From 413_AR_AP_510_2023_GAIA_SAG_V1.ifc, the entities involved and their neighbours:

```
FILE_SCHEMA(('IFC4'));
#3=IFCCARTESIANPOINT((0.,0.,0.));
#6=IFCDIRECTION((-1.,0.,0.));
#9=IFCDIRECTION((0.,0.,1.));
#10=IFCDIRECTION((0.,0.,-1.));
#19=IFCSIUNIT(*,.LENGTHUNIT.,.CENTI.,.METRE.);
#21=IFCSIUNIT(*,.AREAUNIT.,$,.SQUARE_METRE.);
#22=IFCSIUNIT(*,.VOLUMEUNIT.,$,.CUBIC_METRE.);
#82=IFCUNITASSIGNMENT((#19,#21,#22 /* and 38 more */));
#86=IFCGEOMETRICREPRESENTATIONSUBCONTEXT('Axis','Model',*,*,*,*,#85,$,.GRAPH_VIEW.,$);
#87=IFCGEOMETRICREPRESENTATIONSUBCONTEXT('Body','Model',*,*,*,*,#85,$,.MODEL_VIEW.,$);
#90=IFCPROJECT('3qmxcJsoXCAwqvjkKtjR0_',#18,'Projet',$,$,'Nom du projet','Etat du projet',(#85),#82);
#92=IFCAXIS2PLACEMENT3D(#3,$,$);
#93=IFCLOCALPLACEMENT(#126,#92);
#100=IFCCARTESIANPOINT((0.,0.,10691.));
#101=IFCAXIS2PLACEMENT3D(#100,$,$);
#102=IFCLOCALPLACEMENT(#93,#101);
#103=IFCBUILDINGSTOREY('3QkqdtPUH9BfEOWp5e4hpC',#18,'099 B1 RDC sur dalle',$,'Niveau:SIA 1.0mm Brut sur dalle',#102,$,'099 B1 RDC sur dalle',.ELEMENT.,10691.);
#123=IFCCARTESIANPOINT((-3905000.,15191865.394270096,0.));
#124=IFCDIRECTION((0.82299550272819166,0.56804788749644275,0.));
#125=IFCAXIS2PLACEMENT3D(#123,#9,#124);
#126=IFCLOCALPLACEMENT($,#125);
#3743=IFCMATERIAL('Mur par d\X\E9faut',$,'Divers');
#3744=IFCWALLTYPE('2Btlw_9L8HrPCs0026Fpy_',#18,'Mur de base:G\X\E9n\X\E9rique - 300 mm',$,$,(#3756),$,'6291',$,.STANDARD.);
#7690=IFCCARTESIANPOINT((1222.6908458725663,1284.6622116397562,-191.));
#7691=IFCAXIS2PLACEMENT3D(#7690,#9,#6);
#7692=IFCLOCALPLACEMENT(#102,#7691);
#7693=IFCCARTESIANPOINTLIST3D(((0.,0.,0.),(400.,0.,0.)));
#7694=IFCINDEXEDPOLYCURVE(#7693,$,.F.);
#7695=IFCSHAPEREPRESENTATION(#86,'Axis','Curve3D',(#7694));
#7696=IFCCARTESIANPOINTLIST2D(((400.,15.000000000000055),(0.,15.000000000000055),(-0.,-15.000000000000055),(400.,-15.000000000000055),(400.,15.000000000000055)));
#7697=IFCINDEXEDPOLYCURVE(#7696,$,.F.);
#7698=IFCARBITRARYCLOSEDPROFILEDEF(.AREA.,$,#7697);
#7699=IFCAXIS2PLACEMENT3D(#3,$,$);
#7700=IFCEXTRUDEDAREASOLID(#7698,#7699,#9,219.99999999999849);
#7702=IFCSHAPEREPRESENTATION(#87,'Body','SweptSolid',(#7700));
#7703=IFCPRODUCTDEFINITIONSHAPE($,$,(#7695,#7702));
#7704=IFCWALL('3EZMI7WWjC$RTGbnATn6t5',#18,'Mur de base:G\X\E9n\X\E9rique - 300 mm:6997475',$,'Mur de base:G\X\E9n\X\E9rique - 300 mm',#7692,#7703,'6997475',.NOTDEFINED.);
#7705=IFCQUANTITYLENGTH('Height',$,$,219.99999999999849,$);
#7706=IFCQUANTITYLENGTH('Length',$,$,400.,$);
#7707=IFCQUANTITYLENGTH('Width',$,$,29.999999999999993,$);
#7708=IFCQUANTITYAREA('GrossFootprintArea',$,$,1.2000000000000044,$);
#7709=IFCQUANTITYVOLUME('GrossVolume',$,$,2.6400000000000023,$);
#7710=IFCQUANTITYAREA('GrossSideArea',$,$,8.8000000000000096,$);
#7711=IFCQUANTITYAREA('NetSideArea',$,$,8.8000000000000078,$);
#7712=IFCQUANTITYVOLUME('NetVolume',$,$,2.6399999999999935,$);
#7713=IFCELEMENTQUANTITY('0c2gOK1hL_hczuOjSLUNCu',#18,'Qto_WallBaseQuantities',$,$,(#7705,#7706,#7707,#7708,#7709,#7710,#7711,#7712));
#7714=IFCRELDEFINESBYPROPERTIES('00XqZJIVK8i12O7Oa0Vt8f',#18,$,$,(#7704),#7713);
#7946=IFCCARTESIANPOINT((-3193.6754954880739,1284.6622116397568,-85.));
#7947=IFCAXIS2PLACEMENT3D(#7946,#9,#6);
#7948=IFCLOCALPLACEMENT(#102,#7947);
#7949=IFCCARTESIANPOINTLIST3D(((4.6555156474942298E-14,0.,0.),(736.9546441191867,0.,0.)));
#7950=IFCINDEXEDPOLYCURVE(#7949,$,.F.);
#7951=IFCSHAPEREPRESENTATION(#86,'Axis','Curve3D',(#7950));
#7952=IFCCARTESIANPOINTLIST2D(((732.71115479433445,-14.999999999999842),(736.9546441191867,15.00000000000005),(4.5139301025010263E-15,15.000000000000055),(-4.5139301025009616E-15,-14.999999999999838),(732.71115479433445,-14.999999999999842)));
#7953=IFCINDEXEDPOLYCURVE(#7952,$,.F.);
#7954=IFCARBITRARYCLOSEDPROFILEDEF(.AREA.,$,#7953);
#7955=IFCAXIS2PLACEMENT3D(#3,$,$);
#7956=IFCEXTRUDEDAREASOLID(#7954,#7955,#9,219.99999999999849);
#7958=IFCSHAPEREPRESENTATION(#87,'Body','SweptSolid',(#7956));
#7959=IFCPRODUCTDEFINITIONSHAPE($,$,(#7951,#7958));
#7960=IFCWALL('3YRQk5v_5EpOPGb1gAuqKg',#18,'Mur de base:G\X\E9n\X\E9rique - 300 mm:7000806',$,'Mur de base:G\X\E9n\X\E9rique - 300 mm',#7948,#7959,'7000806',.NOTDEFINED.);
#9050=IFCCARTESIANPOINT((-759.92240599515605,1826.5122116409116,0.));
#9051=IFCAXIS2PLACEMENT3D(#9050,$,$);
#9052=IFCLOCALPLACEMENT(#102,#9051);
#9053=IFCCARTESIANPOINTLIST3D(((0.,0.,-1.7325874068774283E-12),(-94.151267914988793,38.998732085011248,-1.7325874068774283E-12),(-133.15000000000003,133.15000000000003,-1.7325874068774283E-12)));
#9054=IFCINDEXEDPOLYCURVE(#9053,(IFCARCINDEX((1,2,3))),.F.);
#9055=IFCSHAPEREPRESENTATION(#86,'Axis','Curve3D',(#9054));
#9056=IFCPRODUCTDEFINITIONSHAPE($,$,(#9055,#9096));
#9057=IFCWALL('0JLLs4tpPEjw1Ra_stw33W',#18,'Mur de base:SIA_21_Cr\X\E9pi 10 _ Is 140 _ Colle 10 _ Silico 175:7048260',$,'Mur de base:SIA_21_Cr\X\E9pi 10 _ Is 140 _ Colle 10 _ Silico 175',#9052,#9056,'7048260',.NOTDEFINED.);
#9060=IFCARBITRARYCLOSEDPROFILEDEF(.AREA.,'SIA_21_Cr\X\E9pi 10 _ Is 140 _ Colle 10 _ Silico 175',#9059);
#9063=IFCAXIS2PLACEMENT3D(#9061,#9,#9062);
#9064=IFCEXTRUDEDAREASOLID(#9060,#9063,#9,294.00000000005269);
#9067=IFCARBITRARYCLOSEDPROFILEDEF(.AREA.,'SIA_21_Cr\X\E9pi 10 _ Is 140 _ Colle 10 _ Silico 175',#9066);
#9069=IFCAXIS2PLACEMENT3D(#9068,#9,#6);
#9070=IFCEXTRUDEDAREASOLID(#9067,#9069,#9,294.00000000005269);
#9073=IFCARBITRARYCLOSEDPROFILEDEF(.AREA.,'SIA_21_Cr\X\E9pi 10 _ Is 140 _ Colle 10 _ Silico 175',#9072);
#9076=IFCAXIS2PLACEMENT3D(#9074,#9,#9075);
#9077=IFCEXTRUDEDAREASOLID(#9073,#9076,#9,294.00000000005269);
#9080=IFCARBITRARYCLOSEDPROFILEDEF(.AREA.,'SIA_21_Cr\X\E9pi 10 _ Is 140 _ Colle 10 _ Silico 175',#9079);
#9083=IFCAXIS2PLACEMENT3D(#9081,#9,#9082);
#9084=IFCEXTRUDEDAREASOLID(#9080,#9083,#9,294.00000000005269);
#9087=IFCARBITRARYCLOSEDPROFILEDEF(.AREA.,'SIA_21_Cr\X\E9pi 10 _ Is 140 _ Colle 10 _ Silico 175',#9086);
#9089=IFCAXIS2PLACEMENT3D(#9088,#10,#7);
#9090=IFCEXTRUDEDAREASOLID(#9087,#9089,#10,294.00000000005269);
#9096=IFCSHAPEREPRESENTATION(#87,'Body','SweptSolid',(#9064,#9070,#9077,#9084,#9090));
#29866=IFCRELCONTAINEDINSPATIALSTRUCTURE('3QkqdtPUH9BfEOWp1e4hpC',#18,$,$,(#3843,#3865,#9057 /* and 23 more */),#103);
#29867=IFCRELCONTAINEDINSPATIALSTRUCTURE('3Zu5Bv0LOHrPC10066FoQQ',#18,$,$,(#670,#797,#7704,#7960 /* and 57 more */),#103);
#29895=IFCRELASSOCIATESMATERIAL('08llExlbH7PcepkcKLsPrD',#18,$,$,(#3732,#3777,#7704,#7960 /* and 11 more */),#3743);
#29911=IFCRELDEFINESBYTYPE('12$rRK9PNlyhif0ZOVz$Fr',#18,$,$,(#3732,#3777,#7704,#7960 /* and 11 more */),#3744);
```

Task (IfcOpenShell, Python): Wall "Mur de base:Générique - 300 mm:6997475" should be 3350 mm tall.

```python
import ifcopenshell
import ifcopenshell.api.pset
import ifcopenshell.geom
import ifcopenshell.util.element
import ifcopenshell.util.representation
import ifcopenshell.util.shape
import ifcopenshell.util.unit

model = ifcopenshell.open("413_AR_AP_510_2023_GAIA_SAG_V1.ifc")
unit_scale = ifcopenshell.util.unit.calculate_unit_scale(model)
area_scale = ifcopenshell.util.unit.calculate_unit_scale(model, "AREAUNIT")
volume_scale = ifcopenshell.util.unit.calculate_unit_scale(model, "VOLUMEUNIT")
settings = ifcopenshell.geom.settings()


def volume(element):
    """Net volume in cubic metres, openings subtracted."""
    shape = ifcopenshell.geom.create_shape(settings, element)
    return ifcopenshell.util.shape.get_volume(shape.geometry)


wall = model.by_guid("3EZMI7WWjC$RTGbnATn6t5")
before = volume(wall)

body = ifcopenshell.util.representation.get_representation(wall, "Model", "Body")
solid = body.Items[0]
old_height = solid.Depth
solid.Depth = 3.35 / unit_scale
after = volume(wall)
thickness = 0.3  # wall thickness in metres

# Update the stored height, areas and volumes.
qto = model.by_id(ifcopenshell.util.element.get_pset(wall, "Qto_WallBaseQuantities", should_inherit=False)["id"])
ifcopenshell.api.pset.edit_qto(model, qto=qto, properties={
    "Height": solid.Depth,
    "GrossVolume": ifcopenshell.util.element.get_pset(wall, "Qto_WallBaseQuantities", "GrossVolume") * solid.Depth / old_height,
    "GrossSideArea": ifcopenshell.util.element.get_pset(wall, "Qto_WallBaseQuantities", "GrossSideArea") * solid.Depth / old_height,
    "NetSideArea": after / thickness / area_scale,
    "NetVolume": after / volume_scale,
})

print(f"height {old_height:g} -> {solid.Depth:g}, volume {before:.3f} -> {after:.3f} m3")

model.write("413_AR_AP_510_2023_GAIA_SAG_V1_v2.ifc")
```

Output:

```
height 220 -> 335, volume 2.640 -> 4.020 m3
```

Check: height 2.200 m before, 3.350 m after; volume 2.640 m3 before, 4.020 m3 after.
